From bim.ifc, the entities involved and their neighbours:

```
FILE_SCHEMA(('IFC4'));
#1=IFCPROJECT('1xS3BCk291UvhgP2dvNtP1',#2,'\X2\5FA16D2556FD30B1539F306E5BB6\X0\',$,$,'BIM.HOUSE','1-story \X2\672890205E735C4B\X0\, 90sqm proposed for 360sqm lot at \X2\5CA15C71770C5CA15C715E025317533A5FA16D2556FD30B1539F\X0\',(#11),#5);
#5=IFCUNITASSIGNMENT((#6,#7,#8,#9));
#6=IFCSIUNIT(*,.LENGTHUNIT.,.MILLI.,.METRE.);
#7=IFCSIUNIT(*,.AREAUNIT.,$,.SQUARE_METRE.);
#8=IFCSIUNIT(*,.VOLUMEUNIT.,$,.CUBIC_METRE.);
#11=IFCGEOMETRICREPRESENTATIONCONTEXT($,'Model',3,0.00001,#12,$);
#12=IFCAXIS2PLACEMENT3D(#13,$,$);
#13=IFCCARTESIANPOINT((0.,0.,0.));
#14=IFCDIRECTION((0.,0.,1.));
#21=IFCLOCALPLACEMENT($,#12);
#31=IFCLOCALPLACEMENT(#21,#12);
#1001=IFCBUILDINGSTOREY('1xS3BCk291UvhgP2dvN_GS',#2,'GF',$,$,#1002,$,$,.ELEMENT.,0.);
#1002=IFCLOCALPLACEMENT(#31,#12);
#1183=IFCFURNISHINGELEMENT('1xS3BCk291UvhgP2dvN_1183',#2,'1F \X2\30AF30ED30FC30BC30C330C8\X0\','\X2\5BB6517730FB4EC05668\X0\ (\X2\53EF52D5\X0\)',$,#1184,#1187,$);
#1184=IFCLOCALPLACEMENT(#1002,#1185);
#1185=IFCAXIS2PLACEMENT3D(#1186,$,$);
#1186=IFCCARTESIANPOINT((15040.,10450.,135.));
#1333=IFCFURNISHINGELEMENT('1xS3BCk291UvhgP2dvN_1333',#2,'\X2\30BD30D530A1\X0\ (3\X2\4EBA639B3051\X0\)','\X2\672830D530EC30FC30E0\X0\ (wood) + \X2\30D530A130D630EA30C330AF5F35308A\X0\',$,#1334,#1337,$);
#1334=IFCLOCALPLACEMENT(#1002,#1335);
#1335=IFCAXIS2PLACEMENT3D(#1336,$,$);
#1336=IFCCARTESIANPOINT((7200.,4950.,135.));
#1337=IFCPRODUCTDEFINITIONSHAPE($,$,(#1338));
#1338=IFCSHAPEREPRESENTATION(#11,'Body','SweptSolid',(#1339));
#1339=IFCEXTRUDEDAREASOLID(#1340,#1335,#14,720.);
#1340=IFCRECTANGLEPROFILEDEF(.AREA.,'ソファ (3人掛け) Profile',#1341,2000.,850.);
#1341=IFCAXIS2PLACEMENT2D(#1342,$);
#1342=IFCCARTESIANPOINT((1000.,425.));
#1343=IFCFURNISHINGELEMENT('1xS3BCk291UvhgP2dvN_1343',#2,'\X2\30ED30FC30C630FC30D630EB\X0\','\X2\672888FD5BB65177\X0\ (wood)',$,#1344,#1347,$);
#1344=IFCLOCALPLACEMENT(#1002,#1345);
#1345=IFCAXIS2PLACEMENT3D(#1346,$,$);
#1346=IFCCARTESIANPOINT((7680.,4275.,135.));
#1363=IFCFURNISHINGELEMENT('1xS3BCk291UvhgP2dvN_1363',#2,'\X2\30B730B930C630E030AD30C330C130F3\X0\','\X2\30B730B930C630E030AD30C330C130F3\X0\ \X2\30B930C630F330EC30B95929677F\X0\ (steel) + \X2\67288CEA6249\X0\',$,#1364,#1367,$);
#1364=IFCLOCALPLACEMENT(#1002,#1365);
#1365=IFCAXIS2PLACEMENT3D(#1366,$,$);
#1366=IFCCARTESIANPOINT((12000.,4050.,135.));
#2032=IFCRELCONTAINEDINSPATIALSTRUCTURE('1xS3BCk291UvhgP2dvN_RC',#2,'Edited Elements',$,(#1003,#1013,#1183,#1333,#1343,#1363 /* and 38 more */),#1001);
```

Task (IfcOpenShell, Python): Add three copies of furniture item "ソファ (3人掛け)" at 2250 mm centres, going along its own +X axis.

```python
import ifcopenshell
import ifcopenshell.api.geometry
import ifcopenshell.api.root
import ifcopenshell.util.element
import ifcopenshell.util.placement

model = ifcopenshell.open("bim.ifc")


def reuse_history(source, copy):
    """copy_class also copies each property set's owner history, people and application; keep the originals."""
    for rel in copy.IsDefinedBy:
        if rel.is_a("IfcRelDefinesByProperties") and (history := rel.RelatingPropertyDefinition.OwnerHistory):
            rel.RelatingPropertyDefinition.OwnerHistory = source.OwnerHistory
            ifcopenshell.util.element.remove_deep2(model, history)


source = model.by_id(1333)
base = ifcopenshell.util.placement.get_local_placement(source.ObjectPlacement)
step = base[:3, 0] * 2250.0

for i in range(1, 4):
    copy = ifcopenshell.api.root.copy_class(model, product=source)
    copy.Representation = ifcopenshell.util.element.copy_deep(
        model, source.Representation, exclude=["IfcGeometricRepresentationContext", "IfcRepresentationMap"]
    )
    reuse_history(source, copy)
    matrix = base.copy()
    matrix[:3, 3] += i * step
    print("added at", matrix[:3, 3].round(3) + 0.0)
    ifcopenshell.api.geometry.edit_object_placement(model, product=copy, matrix=matrix, is_si=False)

model.write("bim_edited.ifc")
```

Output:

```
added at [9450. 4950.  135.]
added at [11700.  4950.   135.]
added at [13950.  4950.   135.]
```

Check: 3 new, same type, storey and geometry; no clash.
